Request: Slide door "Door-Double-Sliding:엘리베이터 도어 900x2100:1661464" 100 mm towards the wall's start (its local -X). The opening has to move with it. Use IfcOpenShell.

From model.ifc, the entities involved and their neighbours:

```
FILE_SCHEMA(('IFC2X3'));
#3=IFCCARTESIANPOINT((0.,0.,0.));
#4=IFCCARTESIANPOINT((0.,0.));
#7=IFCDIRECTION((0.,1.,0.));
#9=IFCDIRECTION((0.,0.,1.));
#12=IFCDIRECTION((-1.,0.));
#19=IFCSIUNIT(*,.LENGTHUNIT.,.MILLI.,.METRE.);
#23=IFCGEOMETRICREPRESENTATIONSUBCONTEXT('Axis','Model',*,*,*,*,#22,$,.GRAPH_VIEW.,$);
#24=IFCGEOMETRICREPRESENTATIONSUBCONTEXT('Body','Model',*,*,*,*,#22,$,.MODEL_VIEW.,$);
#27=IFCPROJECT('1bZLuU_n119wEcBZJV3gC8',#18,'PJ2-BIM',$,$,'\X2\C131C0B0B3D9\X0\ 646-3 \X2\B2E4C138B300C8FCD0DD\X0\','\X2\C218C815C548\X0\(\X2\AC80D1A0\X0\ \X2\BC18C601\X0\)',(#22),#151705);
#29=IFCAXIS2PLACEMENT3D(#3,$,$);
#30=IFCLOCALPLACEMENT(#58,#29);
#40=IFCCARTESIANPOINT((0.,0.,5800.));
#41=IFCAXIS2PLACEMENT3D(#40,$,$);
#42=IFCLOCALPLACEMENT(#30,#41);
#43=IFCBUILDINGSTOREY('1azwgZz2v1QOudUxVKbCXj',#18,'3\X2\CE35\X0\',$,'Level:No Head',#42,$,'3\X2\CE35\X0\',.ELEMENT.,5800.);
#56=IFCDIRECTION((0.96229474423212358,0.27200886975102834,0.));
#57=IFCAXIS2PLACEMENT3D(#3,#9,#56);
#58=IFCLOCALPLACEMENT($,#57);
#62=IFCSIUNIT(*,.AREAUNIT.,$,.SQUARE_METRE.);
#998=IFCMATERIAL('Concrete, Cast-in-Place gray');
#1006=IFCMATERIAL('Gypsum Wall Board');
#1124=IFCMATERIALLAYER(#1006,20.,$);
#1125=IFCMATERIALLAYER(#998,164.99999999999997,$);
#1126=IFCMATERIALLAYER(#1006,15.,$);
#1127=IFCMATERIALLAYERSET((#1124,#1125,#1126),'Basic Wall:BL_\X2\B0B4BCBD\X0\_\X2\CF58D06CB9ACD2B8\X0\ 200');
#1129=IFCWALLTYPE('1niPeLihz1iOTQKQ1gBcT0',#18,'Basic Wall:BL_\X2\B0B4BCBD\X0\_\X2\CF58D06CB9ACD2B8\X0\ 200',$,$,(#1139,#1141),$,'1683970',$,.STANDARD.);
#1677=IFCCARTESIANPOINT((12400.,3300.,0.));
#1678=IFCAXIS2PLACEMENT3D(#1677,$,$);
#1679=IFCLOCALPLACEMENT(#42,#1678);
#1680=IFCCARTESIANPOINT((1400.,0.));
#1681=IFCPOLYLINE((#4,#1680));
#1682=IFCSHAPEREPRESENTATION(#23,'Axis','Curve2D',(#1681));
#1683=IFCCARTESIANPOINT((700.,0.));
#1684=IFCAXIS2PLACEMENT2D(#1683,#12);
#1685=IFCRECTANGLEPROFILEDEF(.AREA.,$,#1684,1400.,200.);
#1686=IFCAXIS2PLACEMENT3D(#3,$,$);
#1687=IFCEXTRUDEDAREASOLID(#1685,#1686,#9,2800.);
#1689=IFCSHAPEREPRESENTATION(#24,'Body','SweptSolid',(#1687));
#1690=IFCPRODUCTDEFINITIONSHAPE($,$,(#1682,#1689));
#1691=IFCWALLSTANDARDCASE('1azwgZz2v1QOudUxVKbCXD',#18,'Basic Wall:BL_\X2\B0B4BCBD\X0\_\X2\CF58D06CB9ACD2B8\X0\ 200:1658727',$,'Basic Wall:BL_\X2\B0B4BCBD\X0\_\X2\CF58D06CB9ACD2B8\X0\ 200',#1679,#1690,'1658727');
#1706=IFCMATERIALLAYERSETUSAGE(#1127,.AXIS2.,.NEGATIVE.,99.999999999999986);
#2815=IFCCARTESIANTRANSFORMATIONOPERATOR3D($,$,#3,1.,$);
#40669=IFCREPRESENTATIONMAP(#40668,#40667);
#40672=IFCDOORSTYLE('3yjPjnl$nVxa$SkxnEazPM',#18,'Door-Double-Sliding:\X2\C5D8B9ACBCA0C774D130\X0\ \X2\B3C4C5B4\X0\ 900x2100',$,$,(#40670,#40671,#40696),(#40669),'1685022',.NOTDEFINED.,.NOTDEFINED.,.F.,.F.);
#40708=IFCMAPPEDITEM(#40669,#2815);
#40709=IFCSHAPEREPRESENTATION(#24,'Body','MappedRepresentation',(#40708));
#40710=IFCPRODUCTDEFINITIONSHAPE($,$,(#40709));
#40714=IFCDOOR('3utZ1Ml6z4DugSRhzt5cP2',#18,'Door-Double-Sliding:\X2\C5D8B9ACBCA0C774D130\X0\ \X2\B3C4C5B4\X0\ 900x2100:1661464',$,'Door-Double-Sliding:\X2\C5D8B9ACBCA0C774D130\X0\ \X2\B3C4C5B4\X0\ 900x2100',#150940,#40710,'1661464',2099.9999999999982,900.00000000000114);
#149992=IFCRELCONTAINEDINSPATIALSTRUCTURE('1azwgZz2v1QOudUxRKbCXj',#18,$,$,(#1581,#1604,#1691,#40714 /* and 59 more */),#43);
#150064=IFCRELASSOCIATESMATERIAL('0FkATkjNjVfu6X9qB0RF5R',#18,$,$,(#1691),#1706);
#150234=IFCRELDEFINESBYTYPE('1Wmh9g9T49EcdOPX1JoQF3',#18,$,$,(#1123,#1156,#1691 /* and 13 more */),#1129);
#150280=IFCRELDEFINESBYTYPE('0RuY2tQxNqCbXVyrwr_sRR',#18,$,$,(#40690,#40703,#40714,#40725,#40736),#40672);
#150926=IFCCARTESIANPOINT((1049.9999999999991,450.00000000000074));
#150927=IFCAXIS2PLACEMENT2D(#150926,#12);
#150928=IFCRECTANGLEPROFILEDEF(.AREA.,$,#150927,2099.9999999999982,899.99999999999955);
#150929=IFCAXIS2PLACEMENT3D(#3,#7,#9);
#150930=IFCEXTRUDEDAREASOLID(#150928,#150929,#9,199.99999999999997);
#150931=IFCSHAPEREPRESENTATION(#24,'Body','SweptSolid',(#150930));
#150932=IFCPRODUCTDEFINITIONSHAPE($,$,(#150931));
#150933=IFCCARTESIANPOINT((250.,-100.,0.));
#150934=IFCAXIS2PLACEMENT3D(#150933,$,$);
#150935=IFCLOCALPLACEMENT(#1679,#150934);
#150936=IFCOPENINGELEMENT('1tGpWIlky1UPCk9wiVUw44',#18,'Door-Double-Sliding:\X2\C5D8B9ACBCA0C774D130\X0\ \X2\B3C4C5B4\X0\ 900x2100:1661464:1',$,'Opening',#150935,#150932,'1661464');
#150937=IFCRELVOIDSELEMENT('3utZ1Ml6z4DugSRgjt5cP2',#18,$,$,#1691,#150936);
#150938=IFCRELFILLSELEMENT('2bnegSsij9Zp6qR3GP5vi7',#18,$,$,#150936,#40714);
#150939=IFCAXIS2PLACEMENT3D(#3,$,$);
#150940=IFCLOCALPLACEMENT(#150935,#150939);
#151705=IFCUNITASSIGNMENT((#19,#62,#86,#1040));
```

```python
import ifcopenshell
import ifcopenshell.api.geometry
import ifcopenshell.util.placement
import ifcopenshell.util.unit

model = ifcopenshell.open("model.ifc")
unit_scale = ifcopenshell.util.unit.calculate_unit_scale(model)

door = model.by_guid("3utZ1Ml6z4DugSRhzt5cP2")
opening = door.FillsVoids[0].RelatingOpeningElement
wall = opening.VoidsElements[0].RelatingBuildingElement

wall_matrix = ifcopenshell.util.placement.get_local_placement(wall.ObjectPlacement)
shift = wall_matrix[:3, 0] * -0.1 / unit_scale
before = ifcopenshell.util.placement.get_local_placement(door.ObjectPlacement)[:3, 3].copy()

# The door is placed relative to its opening, so it follows when the opening moves.
matrix = ifcopenshell.util.placement.get_local_placement(opening.ObjectPlacement)
matrix[:3, 3] += shift
ifcopenshell.api.geometry.edit_object_placement(
    model, product=opening, matrix=matrix, is_si=False, should_transform_children=True
)

after = ifcopenshell.util.placement.get_local_placement(door.ObjectPlacement)[:3, 3]
print("door moved by", (after - before).round(3) + 0.0)

model.write("model-out.ifc")
```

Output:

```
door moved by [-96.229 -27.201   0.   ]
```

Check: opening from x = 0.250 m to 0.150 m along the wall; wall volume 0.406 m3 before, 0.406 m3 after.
